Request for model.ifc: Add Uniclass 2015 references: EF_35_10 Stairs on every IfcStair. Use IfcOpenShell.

First a look at what the model holds.

```python
import ifcopenshell

model = ifcopenshell.open("model.ifc")
print(model.schema)
print("classifications:", [c.Name for c in model.by_type("IfcClassification")])
for ifc_class in ("IfcDoor", "IfcRoof", "IfcStair", "IfcWall", "IfcWindow"):
    print(ifc_class, len(model.by_type(ifc_class)))
```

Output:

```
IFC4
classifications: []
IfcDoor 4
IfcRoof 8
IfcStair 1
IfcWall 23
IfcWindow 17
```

```python
import ifcopenshell
import ifcopenshell.api.classification

model = ifcopenshell.open("model.ifc")

system = ifcopenshell.api.classification.add_classification(model, classification="Uniclass 2015")

codes = {
    "IfcStair": ("EF_35_10", "Stairs"),
}
for ifc_class, (code, name) in codes.items():
    products = model.by_type(ifc_class)
    ifcopenshell.api.classification.add_reference(
        model, products=products, classification=system, identification=code, name=name
    )
    print(code, len(products))

model.write("model-out.ifc")
```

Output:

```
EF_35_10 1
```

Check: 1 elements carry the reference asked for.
